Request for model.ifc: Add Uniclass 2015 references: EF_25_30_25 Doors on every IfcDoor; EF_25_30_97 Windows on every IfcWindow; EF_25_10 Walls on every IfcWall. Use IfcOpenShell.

First a look at what the model holds.

```python
import ifcopenshell

model = ifcopenshell.open("model.ifc")
print(model.schema)
print("classifications:", [c.Name for c in model.by_type("IfcClassification")])
for ifc_class in ("IfcDoor", "IfcRoof", "IfcStair", "IfcWall", "IfcWindow"):
    print(ifc_class, len(model.by_type(ifc_class)))
```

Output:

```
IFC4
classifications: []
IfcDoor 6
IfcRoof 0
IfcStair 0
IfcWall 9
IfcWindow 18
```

```python
import ifcopenshell
import ifcopenshell.api.classification

model = ifcopenshell.open("model.ifc")

system = ifcopenshell.api.classification.add_classification(model, classification="Uniclass 2015")

codes = {
    "IfcDoor": ("EF_25_30_25", "Doors"),
    "IfcWindow": ("EF_25_30_97", "Windows"),
    "IfcWall": ("EF_25_10", "Walls"),
}
for ifc_class, (code, name) in codes.items():
    products = model.by_type(ifc_class)
    ifcopenshell.api.classification.add_reference(
        model, products=products, classification=system, identification=code, name=name
    )
    print(code, len(products))

model.write("model_rev.ifc")
```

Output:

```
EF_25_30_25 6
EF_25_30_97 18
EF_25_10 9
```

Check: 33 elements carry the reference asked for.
